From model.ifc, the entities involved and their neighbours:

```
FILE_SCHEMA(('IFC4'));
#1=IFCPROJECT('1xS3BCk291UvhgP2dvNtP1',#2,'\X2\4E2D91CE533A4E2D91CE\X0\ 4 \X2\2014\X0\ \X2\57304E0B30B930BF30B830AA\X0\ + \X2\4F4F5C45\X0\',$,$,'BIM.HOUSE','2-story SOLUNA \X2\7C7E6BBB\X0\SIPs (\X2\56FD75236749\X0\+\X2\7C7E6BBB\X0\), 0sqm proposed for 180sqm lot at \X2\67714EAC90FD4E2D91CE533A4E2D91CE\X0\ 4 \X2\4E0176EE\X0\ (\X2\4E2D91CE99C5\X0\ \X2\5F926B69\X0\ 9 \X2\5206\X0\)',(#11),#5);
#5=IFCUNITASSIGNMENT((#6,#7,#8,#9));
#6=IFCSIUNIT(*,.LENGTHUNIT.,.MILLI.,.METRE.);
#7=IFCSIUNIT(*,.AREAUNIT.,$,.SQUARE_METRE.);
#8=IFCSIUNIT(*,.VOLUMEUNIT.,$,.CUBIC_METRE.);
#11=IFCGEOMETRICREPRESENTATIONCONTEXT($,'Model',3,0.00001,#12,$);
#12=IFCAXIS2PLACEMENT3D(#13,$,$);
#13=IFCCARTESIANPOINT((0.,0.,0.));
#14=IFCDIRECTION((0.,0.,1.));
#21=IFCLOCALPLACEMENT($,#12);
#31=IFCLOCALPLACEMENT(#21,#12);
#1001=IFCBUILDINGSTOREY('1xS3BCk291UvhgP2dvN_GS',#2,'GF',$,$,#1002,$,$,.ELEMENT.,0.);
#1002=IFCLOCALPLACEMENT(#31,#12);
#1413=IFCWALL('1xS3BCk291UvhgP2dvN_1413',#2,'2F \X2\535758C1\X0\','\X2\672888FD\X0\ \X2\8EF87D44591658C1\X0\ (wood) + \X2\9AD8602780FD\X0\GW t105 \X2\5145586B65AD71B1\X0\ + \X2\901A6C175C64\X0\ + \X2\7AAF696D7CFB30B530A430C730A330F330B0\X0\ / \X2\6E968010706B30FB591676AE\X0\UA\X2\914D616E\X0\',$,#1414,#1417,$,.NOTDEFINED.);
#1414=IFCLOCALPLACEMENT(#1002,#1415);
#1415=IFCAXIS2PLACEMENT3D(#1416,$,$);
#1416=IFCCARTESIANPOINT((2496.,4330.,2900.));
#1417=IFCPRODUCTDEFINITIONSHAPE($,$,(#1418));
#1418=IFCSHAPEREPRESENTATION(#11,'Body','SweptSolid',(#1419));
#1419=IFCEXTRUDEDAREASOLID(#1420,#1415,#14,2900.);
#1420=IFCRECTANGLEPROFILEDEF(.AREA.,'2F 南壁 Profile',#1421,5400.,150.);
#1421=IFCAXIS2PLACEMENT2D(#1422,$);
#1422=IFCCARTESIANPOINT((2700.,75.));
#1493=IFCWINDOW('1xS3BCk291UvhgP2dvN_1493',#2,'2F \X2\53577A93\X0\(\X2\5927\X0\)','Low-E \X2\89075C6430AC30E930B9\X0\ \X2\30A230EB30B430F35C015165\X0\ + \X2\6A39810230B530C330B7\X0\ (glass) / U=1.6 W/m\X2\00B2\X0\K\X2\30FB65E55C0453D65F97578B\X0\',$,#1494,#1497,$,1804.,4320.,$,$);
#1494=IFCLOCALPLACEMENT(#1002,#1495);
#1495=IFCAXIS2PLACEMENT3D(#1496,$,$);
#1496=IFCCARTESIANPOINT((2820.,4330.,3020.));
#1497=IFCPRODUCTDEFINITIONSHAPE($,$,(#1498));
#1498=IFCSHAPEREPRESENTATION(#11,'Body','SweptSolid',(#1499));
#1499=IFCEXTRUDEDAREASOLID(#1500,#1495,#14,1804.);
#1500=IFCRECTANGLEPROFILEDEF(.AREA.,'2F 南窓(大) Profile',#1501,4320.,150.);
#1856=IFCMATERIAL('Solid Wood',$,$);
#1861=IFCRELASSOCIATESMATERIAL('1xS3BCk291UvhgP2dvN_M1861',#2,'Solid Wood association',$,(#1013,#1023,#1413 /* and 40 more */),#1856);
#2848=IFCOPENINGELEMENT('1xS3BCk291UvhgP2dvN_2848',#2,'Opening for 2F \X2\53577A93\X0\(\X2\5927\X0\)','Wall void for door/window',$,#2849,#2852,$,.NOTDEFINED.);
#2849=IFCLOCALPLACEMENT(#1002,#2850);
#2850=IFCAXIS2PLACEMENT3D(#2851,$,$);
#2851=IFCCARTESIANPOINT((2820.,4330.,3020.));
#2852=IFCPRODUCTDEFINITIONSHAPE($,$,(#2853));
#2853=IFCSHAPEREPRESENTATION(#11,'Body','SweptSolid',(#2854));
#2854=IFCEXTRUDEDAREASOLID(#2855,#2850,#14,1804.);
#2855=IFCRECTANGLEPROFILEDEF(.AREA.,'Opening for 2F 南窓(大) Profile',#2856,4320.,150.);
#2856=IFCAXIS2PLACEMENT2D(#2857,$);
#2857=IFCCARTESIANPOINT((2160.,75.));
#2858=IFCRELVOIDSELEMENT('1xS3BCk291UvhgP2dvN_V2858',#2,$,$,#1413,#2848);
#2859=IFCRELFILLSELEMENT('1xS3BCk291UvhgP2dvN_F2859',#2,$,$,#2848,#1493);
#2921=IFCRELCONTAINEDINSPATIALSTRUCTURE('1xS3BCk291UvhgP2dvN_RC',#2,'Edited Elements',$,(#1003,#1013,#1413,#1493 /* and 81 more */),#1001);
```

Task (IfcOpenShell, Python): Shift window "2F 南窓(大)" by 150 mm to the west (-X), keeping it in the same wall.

```python
import ifcopenshell
import ifcopenshell.api.geometry
import ifcopenshell.util.placement
import ifcopenshell.util.unit

model = ifcopenshell.open("model.ifc")
unit_scale = ifcopenshell.util.unit.calculate_unit_scale(model)

window = model.by_id(1493)
opening = window.FillsVoids[0].RelatingOpeningElement
wall = opening.VoidsElements[0].RelatingBuildingElement

wall_matrix = ifcopenshell.util.placement.get_local_placement(wall.ObjectPlacement)
shift = wall_matrix[:3, 0] * -0.15 / unit_scale
before = ifcopenshell.util.placement.get_local_placement(window.ObjectPlacement)[:3, 3].copy()

# The window is not placed relative to its opening, so move both.
for product in (opening, window):
    matrix = ifcopenshell.util.placement.get_local_placement(product.ObjectPlacement)
    matrix[:3, 3] += shift
    ifcopenshell.api.geometry.edit_object_placement(model, product=product, matrix=matrix, is_si=False)

after = ifcopenshell.util.placement.get_local_placement(window.ObjectPlacement)[:3, 3]
print("window moved by", (after - before).round(3) + 0.0)

model.write("model_rev.ifc")
```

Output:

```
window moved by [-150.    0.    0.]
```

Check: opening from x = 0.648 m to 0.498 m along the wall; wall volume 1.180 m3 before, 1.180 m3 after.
